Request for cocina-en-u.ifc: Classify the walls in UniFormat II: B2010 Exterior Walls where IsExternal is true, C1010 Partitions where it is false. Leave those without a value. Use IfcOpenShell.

First a look at what the model holds.

```python
import ifcopenshell
import ifcopenshell.util.element

model = ifcopenshell.open("cocina-en-u.ifc")
print(model.schema)
print("classifications:", [c.Name for c in model.by_type("IfcClassification")])
values = [ifcopenshell.util.element.get_pset(e, "Pset_WallCommon", "IsExternal") for e in model.by_type("IfcWall")]
for value in (True, False, None):
    print("IsExternal", value, values.count(value))
```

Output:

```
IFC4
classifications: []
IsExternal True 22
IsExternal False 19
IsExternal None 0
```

```python
import ifcopenshell
import ifcopenshell.api.classification
import ifcopenshell.util.element

model = ifcopenshell.open("cocina-en-u.ifc")

system = ifcopenshell.api.classification.add_classification(model, classification="UniFormat II")

walls = model.by_type("IfcWall")
external = {e: ifcopenshell.util.element.get_pset(e, "Pset_WallCommon", "IsExternal") for e in walls}
for flag, code, name in ((True, "B2010", "Exterior Walls"), (False, "C1010", "Partitions")):
    products = [e for e in walls if external[e] is flag]
    ifcopenshell.api.classification.add_reference(
        model, products=products, classification=system, identification=code, name=name
    )
    print(code, len(products))

model.write("cocina-en-u_v2.ifc")
```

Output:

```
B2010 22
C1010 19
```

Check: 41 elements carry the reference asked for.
